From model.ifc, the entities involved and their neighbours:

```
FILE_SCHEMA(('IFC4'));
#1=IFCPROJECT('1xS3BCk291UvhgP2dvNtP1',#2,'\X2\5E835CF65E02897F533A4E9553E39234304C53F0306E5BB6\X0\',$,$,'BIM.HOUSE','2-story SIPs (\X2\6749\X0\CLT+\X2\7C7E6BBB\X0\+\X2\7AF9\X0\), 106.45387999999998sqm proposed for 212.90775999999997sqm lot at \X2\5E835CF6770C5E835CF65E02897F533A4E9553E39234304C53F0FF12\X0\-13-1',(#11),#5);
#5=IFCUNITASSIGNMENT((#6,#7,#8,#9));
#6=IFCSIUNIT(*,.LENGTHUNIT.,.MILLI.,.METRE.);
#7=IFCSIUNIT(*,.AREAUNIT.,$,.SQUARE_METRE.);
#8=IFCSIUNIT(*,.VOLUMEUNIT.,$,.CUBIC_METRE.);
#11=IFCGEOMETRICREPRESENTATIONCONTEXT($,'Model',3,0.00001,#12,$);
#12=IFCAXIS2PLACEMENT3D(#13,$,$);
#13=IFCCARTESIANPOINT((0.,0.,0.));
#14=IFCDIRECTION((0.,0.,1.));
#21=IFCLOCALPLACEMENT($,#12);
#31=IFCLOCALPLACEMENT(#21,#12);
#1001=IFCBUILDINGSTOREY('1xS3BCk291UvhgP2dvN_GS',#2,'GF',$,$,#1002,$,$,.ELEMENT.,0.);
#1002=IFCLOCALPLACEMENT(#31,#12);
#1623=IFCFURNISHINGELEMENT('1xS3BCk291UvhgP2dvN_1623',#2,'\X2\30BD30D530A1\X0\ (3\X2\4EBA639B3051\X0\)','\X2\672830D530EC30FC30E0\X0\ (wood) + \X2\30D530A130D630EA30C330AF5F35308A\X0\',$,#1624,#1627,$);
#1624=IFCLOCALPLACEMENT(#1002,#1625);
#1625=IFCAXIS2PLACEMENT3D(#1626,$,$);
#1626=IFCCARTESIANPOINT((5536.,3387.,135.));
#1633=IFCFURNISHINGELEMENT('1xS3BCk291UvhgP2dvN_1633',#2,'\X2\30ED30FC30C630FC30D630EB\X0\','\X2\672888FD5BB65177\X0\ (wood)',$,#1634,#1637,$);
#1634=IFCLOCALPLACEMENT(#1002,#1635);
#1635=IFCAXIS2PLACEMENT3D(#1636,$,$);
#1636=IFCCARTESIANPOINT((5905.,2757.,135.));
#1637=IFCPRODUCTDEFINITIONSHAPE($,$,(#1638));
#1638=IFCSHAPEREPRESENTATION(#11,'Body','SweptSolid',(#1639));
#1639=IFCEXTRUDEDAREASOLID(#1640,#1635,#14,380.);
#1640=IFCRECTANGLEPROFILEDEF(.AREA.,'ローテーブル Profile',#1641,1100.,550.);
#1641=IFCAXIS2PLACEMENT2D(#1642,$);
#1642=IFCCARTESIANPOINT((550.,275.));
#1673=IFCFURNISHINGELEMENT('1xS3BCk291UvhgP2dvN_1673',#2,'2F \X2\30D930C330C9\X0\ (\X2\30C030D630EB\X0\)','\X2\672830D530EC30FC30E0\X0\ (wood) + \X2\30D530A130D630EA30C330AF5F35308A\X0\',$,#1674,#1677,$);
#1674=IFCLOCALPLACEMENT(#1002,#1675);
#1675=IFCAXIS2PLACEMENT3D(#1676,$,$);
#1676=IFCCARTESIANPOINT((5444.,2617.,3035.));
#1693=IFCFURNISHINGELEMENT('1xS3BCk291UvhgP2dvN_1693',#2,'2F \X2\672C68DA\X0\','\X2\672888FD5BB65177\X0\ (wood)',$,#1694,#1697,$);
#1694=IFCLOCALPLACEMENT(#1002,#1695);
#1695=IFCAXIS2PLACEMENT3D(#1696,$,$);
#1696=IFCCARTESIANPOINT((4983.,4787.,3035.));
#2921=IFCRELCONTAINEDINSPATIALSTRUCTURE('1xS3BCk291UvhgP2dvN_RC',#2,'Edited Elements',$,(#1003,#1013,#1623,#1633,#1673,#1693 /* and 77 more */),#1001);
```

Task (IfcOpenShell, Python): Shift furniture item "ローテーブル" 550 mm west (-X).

```python
import ifcopenshell
import ifcopenshell.api.geometry
import ifcopenshell.util.placement

model = ifcopenshell.open("model.ifc")

item = model.by_guid("1xS3BCk291UvhgP2dvN_1633")
matrix = ifcopenshell.util.placement.get_local_placement(item.ObjectPlacement)
matrix[0, 3] -= 550.0
ifcopenshell.api.geometry.edit_object_placement(model, product=item, matrix=matrix, is_si=False)

print(ifcopenshell.util.placement.get_local_placement(item.ObjectPlacement).round(3) + 0.0)

model.write("model_rev.ifc")
```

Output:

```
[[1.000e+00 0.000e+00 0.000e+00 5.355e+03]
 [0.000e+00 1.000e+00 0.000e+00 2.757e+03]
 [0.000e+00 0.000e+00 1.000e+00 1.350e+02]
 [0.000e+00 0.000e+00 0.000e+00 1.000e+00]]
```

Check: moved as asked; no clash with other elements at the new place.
